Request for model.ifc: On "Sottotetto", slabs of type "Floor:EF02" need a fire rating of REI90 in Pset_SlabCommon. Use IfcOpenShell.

First a look at what the model holds.

```python
import ifcopenshell
import ifcopenshell.util.element

model = ifcopenshell.open("model.ifc")
print(model.schema)
storey = next(s for s in model.by_type("IfcBuildingStorey") if s.Name == "Sottotetto")
slabs = [e for e in ifcopenshell.util.element.get_decomposition(storey) if e.is_a("IfcSlab")]
seen = {}
for e in slabs:
    element_type = ifcopenshell.util.element.get_type(e)
    key = (element_type.Name if element_type != e and element_type else None, ifcopenshell.util.element.get_pset(e, "Pset_SlabCommon", "FireRating"))
    seen[key] = seen.get(key, 0) + 1
for (name, value), count in sorted(seen.items(), key=str):
    print(count, "x", name, "|", value)
```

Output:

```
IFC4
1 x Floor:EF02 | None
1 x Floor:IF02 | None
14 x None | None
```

```python
import ifcopenshell
import ifcopenshell.api.pset
import ifcopenshell.util.element

model = ifcopenshell.open("model.ifc")

storey = next(s for s in model.by_type("IfcBuildingStorey") if s.Name == "Sottotetto")
slabs = [e for e in ifcopenshell.util.element.get_decomposition(storey) if e.is_a("IfcSlab")]

count = 0
for e in slabs:
    element_type = ifcopenshell.util.element.get_type(e)
    if element_type in (None, e) or element_type.Name != "Floor:EF02":
        continue
    # add_pset returns the element's existing set when there is one.
    pset = ifcopenshell.api.pset.add_pset(model, product=e, name="Pset_SlabCommon")
    ifcopenshell.api.pset.edit_pset(model, pset=pset, properties={"FireRating": "REI90"})
    count += 1

print(count, "slabs updated")

model.write("model_edited.ifc")
```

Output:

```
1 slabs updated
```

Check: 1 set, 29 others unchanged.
